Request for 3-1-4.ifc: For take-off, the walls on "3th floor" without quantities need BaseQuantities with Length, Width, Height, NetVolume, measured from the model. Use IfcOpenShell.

First a look at what the model holds.

```python
import ifcopenshell
import ifcopenshell.util.element
import ifcopenshell.util.unit

model = ifcopenshell.open("3-1-4.ifc")
print(model.schema)
for unit_type in ("LENGTHUNIT", "AREAUNIT", "VOLUMEUNIT"):
    print(unit_type, ifcopenshell.util.unit.calculate_unit_scale(model, unit_type))
storey = next(s for s in model.by_type("IfcBuildingStorey") if s.Name == "3th floor")
walls = [e for e in ifcopenshell.util.element.get_decomposition(storey) if e.is_a("IfcWall")]
for e in sorted(walls, key=lambda e: e.id()):
    print(e.id(), e.is_a(), e.Name, list(ifcopenshell.util.element.get_psets(e, qtos_only=True)), sep=" | ")
```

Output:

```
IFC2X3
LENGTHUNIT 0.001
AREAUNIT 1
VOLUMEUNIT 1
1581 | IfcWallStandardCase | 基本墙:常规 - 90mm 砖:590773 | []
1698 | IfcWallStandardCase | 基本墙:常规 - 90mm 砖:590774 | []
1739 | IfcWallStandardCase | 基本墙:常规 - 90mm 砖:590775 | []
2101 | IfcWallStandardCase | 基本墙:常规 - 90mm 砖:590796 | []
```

```python
import ifcopenshell
import ifcopenshell.api.pset
import ifcopenshell.geom
import ifcopenshell.util.element
import ifcopenshell.util.shape
import ifcopenshell.util.unit

model = ifcopenshell.open("3-1-4.ifc")
unit_scale = ifcopenshell.util.unit.calculate_unit_scale(model)
volume_scale = ifcopenshell.util.unit.calculate_unit_scale(model, "VOLUMEUNIT")
settings = ifcopenshell.geom.settings()

storey = next(s for s in model.by_type("IfcBuildingStorey") if s.Name == "3th floor")
walls = [e for e in ifcopenshell.util.element.get_decomposition(storey) if e.is_a("IfcWall")]

for e in sorted(walls, key=lambda e: e.id()):
    if ifcopenshell.util.element.get_psets(e, qtos_only=True, should_inherit=False):
        continue
    # Geometry comes back in metres, in the element's own axes.
    shape = ifcopenshell.geom.create_shape(settings, e)
    values = {
        "Length": ifcopenshell.util.shape.get_x(shape.geometry) / unit_scale,
        "Width": ifcopenshell.util.shape.get_y(shape.geometry) / unit_scale,
        "Height": ifcopenshell.util.shape.get_z(shape.geometry) / unit_scale,
        "NetVolume": ifcopenshell.util.shape.get_volume(shape.geometry) / volume_scale,
    }
    qto = ifcopenshell.api.pset.add_qto(model, product=e, name="BaseQuantities")
    ifcopenshell.api.pset.edit_qto(model, qto=qto, properties=values)
    print(e.id(), {k: round(v, 3) for k, v in values.items()})

model.write("3-1-4_rev.ifc")
```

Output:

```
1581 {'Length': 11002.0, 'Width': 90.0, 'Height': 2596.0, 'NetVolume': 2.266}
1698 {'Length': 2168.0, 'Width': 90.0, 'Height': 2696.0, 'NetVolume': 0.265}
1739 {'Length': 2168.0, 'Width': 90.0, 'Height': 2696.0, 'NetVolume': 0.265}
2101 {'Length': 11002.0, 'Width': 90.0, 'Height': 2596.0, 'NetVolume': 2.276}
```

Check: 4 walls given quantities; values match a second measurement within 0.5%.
